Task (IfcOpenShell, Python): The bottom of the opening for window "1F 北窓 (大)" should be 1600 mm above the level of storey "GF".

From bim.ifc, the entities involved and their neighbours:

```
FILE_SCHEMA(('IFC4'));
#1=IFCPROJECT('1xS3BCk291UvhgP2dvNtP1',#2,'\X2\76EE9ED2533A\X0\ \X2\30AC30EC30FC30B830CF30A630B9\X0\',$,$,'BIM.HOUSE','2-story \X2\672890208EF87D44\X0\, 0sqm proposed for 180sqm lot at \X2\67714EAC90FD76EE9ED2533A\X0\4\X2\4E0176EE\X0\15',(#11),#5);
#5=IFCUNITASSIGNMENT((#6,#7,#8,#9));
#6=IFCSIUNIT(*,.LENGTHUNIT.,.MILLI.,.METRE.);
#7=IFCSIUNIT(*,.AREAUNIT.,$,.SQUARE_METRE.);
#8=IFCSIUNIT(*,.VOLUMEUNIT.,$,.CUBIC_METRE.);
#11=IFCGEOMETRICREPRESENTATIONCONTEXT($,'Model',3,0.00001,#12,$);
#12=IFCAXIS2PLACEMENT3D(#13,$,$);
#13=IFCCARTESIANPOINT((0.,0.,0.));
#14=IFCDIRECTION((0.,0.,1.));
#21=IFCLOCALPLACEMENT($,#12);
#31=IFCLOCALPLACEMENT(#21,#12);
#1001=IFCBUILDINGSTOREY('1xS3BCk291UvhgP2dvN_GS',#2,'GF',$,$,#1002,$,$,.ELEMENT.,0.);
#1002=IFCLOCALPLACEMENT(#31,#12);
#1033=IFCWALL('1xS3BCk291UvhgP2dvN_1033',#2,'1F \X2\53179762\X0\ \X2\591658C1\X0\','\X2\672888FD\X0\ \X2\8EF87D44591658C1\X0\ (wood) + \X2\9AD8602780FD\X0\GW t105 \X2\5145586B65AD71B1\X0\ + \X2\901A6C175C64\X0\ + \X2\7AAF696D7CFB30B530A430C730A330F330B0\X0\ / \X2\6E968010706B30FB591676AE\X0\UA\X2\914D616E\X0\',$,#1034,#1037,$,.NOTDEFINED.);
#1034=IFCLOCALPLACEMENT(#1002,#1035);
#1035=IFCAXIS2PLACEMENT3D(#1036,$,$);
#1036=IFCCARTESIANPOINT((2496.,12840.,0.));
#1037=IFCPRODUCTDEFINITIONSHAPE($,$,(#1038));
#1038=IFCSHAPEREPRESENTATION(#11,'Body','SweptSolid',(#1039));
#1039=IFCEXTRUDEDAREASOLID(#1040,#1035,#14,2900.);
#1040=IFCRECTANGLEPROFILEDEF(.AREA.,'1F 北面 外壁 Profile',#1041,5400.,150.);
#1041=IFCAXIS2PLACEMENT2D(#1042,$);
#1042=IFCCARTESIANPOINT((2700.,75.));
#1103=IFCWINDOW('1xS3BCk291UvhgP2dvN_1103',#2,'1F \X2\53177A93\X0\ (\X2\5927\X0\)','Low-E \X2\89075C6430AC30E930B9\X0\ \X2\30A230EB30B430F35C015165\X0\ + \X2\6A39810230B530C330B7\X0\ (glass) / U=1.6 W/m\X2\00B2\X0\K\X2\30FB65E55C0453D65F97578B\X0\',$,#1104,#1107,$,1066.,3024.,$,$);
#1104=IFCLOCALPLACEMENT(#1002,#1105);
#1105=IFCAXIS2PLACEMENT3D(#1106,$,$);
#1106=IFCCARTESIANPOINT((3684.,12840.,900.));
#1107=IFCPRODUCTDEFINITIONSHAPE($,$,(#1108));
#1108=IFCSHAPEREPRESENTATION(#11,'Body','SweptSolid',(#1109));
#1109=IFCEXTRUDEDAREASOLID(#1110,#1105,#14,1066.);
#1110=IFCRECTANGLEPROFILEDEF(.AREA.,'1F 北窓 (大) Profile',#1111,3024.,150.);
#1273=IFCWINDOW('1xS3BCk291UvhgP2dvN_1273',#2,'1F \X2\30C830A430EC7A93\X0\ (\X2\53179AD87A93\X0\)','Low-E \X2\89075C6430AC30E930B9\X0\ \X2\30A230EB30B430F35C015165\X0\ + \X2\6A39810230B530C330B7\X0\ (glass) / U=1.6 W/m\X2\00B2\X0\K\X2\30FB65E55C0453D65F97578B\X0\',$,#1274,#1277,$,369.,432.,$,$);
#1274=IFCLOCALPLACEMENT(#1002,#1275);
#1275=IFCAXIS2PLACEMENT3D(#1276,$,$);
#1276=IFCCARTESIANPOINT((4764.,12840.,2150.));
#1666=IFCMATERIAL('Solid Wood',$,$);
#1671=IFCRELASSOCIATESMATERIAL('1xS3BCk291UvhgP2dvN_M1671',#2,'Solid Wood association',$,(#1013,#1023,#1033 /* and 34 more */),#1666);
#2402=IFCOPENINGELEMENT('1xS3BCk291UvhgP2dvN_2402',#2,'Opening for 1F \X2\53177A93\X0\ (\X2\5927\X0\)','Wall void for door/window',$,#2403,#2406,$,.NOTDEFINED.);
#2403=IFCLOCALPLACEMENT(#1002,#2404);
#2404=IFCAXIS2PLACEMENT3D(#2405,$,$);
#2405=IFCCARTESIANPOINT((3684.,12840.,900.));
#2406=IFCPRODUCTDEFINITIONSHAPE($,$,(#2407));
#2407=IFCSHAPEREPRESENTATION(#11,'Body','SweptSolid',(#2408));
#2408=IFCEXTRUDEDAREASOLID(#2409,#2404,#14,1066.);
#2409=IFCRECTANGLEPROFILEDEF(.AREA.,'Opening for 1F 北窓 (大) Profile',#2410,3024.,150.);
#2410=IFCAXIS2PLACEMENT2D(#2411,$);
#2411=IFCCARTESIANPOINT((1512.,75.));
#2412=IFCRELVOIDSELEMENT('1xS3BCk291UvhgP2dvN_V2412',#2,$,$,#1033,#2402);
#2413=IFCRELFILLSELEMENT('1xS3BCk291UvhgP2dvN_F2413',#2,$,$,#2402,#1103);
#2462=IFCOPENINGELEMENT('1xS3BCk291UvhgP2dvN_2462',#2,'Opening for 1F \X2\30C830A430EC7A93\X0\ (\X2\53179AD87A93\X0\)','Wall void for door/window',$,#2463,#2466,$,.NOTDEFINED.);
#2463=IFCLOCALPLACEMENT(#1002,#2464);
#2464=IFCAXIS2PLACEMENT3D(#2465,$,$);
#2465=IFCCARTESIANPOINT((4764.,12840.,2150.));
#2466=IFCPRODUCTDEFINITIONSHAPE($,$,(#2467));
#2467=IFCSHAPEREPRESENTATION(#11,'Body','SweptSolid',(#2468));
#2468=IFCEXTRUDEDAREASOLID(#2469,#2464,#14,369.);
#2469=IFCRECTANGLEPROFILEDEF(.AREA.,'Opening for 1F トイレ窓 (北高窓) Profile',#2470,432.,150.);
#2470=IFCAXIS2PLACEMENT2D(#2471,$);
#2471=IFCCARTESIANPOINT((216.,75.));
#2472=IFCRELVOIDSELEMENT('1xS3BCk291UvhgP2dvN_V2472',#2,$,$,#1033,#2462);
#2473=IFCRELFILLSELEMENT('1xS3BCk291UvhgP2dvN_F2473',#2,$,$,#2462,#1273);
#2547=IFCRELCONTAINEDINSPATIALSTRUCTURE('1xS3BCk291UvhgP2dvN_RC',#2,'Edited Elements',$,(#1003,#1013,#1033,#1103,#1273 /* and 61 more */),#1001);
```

```python
import numpy as np
import ifcopenshell
import ifcopenshell.api.geometry
import ifcopenshell.geom
import ifcopenshell.util.element
import ifcopenshell.util.placement
import ifcopenshell.util.shape
import ifcopenshell.util.unit

model = ifcopenshell.open("bim.ifc")
unit_scale = ifcopenshell.util.unit.calculate_unit_scale(model)

window = model.by_id(1103)
opening = window.FillsVoids[0].RelatingOpeningElement
storey = ifcopenshell.util.element.get_container(window, ifc_class="IfcBuildingStorey")
level = ifcopenshell.util.placement.get_local_placement(storey.ObjectPlacement)[2, 3]

# The opening's origin need not be at the sill, so measure its lowest point.
shape = ifcopenshell.geom.create_shape(ifcopenshell.geom.settings(), opening)
bottom = ifcopenshell.util.shape.get_shape_bottom_elevation(shape, shape.geometry) / unit_scale
dz = level + 1.6 / unit_scale - bottom

shift = np.array([0.0, 0.0, dz])
# The window is not placed relative to its opening, so move both.
for product in (opening, window):
    matrix = ifcopenshell.util.placement.get_local_placement(product.ObjectPlacement)
    matrix[:3, 3] += shift
    ifcopenshell.api.geometry.edit_object_placement(model, product=product, matrix=matrix, is_si=False)

print(f"moved by {dz * unit_scale:+.3f} m")

model.write("bim_edited.ifc")
```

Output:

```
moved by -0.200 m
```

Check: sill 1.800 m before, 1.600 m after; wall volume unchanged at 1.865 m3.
